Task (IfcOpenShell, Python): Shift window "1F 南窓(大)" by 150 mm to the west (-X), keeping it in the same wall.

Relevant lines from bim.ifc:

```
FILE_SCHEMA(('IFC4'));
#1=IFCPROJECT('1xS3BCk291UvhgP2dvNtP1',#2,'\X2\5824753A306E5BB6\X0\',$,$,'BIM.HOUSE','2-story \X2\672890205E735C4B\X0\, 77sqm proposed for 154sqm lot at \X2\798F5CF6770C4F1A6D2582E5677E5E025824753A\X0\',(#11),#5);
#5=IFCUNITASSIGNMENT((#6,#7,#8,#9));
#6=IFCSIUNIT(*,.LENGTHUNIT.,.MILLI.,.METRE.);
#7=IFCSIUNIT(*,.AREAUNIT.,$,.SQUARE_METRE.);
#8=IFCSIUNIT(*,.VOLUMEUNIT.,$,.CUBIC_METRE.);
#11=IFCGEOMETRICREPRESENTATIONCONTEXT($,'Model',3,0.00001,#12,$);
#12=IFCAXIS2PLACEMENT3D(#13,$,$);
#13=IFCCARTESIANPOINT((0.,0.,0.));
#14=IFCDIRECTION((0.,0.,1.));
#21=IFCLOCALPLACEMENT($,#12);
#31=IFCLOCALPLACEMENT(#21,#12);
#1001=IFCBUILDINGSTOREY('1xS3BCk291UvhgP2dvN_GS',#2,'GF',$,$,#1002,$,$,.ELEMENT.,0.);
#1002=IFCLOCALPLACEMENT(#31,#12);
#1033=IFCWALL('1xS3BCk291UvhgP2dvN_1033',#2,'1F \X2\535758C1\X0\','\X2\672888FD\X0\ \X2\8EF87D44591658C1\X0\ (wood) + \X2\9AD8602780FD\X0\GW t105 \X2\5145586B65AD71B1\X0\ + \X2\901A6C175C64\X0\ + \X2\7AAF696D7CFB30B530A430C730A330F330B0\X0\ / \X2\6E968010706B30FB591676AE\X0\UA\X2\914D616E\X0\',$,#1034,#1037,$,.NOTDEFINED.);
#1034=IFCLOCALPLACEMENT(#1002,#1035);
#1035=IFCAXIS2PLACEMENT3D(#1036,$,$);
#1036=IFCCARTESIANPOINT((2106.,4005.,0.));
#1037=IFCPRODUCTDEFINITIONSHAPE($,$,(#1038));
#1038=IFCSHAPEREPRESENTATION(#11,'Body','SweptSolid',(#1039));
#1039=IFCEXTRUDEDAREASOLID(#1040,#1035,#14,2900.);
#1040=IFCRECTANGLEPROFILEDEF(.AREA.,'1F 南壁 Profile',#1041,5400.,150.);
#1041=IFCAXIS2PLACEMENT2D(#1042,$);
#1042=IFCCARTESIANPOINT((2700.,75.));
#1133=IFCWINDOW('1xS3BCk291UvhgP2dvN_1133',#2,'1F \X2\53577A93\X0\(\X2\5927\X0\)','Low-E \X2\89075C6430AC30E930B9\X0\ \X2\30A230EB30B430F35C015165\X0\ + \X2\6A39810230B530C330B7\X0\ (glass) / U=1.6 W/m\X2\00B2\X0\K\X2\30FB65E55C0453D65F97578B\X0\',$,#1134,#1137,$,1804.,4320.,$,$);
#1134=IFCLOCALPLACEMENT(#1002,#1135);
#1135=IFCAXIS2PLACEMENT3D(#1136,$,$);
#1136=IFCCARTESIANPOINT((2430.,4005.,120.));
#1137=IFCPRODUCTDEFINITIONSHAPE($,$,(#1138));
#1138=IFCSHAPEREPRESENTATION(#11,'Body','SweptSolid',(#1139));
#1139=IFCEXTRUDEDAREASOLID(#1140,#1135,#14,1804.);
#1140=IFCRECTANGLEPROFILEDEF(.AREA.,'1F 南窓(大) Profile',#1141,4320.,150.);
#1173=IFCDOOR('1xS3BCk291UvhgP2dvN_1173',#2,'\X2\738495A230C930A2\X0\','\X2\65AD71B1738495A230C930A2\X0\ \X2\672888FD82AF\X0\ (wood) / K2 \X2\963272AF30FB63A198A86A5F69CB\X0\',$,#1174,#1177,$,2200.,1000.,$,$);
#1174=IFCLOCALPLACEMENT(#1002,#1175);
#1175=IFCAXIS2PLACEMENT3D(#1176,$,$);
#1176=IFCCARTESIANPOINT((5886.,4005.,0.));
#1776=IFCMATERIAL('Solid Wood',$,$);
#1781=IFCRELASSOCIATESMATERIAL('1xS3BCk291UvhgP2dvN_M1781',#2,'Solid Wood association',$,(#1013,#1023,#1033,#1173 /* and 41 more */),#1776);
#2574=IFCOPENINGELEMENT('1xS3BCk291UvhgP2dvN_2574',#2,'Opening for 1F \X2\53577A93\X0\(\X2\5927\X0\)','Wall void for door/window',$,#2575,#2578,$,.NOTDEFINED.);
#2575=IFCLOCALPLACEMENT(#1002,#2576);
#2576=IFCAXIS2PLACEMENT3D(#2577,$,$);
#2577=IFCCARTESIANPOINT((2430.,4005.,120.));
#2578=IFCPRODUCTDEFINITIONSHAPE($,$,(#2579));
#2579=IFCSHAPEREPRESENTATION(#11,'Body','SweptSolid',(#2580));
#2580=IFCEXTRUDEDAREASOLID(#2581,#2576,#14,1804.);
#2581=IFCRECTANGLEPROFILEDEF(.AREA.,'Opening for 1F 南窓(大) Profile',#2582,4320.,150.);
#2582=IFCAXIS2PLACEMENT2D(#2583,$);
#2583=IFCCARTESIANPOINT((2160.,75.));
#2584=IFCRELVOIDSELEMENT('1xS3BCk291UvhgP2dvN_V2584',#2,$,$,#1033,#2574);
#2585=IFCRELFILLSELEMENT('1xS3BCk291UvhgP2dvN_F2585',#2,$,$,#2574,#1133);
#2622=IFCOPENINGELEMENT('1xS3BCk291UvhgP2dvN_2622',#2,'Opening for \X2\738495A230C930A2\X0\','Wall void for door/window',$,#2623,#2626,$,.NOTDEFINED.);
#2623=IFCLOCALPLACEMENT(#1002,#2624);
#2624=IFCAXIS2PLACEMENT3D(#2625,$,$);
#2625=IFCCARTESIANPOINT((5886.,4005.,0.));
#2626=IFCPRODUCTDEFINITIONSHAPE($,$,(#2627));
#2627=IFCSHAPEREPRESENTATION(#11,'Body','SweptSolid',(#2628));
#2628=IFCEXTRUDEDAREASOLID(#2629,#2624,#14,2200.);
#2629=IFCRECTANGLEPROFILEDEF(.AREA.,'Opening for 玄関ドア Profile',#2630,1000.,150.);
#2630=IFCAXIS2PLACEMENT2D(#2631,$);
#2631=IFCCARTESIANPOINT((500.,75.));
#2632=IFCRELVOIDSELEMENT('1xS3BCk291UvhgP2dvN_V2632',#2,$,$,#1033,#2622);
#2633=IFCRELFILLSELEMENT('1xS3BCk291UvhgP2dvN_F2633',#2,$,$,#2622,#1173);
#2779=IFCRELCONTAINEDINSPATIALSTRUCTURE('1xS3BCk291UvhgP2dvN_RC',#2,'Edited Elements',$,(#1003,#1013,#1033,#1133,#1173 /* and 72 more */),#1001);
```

```python
import ifcopenshell
import ifcopenshell.api.geometry
import ifcopenshell.util.placement

model = ifcopenshell.open("bim.ifc")

window = model.by_id(1133)
opening = window.FillsVoids[0].RelatingOpeningElement
wall = opening.VoidsElements[0].RelatingBuildingElement

wall_matrix = ifcopenshell.util.placement.get_local_placement(wall.ObjectPlacement)
shift = wall_matrix[:3, 0] * -150.0
before = ifcopenshell.util.placement.get_local_placement(window.ObjectPlacement)[:3, 3].copy()

# The window is not placed relative to its opening, so move both.
for product in (opening, window):
    matrix = ifcopenshell.util.placement.get_local_placement(product.ObjectPlacement)
    matrix[:3, 3] += shift
    ifcopenshell.api.geometry.edit_object_placement(model, product=product, matrix=matrix, is_si=False)

after = ifcopenshell.util.placement.get_local_placement(window.ObjectPlacement)[:3, 3]
print("window moved by", (after - before).round(3) + 0.0)

model.write("bim_edited.ifc")
```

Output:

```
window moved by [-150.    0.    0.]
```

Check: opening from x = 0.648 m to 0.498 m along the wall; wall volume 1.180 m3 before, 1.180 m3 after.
